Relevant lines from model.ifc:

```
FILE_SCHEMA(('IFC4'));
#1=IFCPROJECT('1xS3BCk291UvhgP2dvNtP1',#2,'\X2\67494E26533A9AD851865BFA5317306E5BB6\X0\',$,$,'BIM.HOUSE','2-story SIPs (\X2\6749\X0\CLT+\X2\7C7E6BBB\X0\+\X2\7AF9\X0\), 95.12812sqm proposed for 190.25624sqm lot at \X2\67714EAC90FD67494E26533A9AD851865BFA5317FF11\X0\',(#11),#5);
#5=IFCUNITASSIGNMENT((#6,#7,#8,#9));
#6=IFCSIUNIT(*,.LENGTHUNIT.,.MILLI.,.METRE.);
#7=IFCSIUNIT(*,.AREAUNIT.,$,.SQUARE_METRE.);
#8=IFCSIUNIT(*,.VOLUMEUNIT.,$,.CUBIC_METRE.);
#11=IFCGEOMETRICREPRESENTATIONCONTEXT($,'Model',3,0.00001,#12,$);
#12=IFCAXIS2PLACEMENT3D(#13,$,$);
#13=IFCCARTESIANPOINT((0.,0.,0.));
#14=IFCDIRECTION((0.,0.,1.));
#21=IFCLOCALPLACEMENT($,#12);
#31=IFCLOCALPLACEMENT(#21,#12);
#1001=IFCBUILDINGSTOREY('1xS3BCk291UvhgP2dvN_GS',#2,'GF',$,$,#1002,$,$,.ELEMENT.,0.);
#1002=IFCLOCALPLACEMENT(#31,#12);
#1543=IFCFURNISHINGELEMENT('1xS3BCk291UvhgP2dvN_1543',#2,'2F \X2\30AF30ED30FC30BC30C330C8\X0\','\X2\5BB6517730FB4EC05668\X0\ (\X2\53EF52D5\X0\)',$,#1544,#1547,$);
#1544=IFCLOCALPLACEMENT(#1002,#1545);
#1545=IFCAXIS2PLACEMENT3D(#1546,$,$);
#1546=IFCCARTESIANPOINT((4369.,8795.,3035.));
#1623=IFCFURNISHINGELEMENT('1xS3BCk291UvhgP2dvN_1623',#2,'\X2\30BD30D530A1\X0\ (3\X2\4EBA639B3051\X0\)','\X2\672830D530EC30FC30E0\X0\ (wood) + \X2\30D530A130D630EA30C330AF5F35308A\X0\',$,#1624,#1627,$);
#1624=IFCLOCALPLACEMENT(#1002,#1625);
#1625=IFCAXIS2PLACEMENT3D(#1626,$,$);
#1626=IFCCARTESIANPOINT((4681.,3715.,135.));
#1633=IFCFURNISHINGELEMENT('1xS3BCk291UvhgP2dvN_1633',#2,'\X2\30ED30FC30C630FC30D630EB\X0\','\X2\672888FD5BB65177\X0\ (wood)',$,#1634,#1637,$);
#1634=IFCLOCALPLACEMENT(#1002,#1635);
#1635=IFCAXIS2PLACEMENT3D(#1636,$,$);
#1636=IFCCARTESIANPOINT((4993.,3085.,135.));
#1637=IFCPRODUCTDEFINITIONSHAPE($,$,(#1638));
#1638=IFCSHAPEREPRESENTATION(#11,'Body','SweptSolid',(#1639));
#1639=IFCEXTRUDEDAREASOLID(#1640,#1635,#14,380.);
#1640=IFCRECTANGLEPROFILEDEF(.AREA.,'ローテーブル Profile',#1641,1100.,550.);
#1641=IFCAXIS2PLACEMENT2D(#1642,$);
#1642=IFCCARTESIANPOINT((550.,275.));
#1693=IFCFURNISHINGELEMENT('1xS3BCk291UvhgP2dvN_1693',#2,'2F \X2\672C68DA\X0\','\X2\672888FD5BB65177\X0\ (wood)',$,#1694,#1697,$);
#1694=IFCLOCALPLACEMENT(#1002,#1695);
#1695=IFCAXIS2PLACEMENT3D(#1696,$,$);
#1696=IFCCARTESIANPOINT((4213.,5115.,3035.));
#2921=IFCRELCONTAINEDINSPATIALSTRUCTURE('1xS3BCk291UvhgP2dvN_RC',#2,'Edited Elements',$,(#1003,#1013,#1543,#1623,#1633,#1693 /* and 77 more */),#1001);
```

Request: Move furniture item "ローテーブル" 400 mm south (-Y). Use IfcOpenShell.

```python
import ifcopenshell
import ifcopenshell.api.geometry
import ifcopenshell.util.placement

model = ifcopenshell.open("model.ifc")

item = model.by_guid("1xS3BCk291UvhgP2dvN_1633")
matrix = ifcopenshell.util.placement.get_local_placement(item.ObjectPlacement)
matrix[1, 3] -= 400.0
ifcopenshell.api.geometry.edit_object_placement(model, product=item, matrix=matrix, is_si=False)

print(ifcopenshell.util.placement.get_local_placement(item.ObjectPlacement).round(3) + 0.0)

model.write("model-out.ifc")
```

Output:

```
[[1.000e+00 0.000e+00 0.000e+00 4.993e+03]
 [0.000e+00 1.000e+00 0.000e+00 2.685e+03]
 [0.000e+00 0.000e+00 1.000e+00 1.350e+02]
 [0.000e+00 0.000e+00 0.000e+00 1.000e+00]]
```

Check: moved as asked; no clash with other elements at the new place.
